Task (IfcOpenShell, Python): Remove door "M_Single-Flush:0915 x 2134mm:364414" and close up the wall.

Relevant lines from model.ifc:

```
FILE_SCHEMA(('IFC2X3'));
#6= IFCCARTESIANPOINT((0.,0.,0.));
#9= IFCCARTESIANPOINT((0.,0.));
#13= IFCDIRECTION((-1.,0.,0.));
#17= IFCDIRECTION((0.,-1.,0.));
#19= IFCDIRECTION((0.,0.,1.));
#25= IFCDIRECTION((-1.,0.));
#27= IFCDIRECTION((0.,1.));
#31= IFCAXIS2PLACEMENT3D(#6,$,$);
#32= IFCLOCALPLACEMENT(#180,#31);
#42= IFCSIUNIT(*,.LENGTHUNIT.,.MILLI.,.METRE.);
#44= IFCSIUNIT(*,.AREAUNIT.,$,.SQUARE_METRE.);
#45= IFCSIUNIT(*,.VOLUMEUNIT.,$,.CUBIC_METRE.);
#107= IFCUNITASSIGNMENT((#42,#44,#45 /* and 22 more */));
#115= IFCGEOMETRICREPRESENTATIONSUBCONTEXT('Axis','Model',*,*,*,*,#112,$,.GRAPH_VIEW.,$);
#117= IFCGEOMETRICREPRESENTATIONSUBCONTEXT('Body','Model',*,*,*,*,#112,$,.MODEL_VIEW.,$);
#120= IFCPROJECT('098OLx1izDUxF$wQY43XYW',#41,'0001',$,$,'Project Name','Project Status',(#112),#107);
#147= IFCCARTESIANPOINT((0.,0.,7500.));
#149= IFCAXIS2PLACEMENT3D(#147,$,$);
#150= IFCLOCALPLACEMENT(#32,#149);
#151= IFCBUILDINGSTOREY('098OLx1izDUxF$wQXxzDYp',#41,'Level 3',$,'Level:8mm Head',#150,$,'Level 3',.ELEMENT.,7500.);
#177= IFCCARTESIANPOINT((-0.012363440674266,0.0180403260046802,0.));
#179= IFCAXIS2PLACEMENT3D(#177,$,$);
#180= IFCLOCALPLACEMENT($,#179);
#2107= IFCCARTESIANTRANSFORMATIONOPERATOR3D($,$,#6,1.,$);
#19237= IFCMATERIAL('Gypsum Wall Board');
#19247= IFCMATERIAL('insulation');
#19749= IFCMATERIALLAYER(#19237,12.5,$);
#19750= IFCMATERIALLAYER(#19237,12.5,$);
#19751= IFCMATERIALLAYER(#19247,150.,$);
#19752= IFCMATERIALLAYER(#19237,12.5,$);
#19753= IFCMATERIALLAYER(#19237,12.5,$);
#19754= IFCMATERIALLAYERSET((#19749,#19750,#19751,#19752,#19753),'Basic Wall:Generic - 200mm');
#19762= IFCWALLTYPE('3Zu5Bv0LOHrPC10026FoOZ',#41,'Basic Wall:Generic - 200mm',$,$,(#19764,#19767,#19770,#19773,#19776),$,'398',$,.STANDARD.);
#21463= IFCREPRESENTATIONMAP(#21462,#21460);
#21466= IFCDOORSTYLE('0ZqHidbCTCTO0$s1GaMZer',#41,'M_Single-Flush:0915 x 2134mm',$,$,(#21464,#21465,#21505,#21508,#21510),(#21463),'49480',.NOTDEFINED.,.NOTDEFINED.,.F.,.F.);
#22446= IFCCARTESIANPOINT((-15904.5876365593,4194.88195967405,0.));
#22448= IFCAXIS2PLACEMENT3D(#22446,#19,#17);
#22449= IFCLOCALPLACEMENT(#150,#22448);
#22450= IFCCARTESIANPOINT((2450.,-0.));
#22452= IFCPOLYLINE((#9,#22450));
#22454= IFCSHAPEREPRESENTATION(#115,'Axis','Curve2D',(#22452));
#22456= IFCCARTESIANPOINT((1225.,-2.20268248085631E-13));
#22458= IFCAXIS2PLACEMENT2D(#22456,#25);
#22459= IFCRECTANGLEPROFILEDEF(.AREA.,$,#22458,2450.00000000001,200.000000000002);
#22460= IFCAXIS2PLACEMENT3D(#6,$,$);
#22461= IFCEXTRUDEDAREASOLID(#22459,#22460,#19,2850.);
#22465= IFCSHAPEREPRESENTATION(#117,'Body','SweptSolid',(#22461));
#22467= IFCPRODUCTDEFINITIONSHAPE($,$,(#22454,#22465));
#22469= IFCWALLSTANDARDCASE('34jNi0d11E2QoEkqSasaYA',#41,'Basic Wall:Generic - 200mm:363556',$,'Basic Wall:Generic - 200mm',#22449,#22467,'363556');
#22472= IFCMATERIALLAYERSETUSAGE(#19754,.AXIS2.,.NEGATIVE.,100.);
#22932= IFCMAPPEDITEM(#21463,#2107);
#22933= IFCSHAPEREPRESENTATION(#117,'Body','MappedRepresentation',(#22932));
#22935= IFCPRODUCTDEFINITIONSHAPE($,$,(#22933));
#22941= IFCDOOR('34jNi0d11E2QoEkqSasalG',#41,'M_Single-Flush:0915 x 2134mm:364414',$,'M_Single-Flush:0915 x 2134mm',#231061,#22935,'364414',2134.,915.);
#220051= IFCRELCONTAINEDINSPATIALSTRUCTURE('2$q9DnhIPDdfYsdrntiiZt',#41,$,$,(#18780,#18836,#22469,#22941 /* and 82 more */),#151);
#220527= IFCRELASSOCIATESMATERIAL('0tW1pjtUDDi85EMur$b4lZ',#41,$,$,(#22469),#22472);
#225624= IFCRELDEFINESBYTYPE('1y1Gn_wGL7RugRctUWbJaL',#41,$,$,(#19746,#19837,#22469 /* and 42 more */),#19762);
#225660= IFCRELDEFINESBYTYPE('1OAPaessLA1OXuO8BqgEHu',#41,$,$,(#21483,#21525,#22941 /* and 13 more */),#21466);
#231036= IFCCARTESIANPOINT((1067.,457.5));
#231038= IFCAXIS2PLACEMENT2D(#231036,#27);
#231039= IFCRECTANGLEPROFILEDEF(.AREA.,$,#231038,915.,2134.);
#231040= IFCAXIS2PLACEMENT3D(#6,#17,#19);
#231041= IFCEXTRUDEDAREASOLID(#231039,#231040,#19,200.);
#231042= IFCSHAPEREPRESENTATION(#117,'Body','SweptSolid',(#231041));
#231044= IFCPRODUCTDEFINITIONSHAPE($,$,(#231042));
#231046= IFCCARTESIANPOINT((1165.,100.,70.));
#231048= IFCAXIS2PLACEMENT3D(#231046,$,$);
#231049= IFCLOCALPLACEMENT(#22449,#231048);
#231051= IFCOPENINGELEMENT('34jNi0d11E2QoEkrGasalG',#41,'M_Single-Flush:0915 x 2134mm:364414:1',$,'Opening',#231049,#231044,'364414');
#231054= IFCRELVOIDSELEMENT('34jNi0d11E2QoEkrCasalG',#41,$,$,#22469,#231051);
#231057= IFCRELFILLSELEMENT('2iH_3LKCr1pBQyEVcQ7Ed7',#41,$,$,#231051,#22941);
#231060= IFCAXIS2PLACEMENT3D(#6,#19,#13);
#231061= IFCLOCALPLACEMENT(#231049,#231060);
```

```python
import ifcopenshell
import ifcopenshell.api.feature
import ifcopenshell.api.root
import ifcopenshell.geom
import ifcopenshell.util.shape

model = ifcopenshell.open("model.ifc")
settings = ifcopenshell.geom.settings()


def volume(element):
    """Net volume in cubic metres, openings subtracted."""
    shape = ifcopenshell.geom.create_shape(settings, element)
    return ifcopenshell.util.shape.get_volume(shape.geometry)


door = model.by_guid("34jNi0d11E2QoEkqSasalG")
opening = door.FillsVoids[0].RelatingOpeningElement
wall = opening.VoidsElements[0].RelatingBuildingElement
before = volume(wall)

ifcopenshell.api.root.remove_product(model, product=door)
ifcopenshell.api.feature.remove_feature(model, feature=opening)

after = volume(wall)

print(f"wall volume {before:.3f} -> {after:.3f} m3")

model.write("model-out.ifc")
```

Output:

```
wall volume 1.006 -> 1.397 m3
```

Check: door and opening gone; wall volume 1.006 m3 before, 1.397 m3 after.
